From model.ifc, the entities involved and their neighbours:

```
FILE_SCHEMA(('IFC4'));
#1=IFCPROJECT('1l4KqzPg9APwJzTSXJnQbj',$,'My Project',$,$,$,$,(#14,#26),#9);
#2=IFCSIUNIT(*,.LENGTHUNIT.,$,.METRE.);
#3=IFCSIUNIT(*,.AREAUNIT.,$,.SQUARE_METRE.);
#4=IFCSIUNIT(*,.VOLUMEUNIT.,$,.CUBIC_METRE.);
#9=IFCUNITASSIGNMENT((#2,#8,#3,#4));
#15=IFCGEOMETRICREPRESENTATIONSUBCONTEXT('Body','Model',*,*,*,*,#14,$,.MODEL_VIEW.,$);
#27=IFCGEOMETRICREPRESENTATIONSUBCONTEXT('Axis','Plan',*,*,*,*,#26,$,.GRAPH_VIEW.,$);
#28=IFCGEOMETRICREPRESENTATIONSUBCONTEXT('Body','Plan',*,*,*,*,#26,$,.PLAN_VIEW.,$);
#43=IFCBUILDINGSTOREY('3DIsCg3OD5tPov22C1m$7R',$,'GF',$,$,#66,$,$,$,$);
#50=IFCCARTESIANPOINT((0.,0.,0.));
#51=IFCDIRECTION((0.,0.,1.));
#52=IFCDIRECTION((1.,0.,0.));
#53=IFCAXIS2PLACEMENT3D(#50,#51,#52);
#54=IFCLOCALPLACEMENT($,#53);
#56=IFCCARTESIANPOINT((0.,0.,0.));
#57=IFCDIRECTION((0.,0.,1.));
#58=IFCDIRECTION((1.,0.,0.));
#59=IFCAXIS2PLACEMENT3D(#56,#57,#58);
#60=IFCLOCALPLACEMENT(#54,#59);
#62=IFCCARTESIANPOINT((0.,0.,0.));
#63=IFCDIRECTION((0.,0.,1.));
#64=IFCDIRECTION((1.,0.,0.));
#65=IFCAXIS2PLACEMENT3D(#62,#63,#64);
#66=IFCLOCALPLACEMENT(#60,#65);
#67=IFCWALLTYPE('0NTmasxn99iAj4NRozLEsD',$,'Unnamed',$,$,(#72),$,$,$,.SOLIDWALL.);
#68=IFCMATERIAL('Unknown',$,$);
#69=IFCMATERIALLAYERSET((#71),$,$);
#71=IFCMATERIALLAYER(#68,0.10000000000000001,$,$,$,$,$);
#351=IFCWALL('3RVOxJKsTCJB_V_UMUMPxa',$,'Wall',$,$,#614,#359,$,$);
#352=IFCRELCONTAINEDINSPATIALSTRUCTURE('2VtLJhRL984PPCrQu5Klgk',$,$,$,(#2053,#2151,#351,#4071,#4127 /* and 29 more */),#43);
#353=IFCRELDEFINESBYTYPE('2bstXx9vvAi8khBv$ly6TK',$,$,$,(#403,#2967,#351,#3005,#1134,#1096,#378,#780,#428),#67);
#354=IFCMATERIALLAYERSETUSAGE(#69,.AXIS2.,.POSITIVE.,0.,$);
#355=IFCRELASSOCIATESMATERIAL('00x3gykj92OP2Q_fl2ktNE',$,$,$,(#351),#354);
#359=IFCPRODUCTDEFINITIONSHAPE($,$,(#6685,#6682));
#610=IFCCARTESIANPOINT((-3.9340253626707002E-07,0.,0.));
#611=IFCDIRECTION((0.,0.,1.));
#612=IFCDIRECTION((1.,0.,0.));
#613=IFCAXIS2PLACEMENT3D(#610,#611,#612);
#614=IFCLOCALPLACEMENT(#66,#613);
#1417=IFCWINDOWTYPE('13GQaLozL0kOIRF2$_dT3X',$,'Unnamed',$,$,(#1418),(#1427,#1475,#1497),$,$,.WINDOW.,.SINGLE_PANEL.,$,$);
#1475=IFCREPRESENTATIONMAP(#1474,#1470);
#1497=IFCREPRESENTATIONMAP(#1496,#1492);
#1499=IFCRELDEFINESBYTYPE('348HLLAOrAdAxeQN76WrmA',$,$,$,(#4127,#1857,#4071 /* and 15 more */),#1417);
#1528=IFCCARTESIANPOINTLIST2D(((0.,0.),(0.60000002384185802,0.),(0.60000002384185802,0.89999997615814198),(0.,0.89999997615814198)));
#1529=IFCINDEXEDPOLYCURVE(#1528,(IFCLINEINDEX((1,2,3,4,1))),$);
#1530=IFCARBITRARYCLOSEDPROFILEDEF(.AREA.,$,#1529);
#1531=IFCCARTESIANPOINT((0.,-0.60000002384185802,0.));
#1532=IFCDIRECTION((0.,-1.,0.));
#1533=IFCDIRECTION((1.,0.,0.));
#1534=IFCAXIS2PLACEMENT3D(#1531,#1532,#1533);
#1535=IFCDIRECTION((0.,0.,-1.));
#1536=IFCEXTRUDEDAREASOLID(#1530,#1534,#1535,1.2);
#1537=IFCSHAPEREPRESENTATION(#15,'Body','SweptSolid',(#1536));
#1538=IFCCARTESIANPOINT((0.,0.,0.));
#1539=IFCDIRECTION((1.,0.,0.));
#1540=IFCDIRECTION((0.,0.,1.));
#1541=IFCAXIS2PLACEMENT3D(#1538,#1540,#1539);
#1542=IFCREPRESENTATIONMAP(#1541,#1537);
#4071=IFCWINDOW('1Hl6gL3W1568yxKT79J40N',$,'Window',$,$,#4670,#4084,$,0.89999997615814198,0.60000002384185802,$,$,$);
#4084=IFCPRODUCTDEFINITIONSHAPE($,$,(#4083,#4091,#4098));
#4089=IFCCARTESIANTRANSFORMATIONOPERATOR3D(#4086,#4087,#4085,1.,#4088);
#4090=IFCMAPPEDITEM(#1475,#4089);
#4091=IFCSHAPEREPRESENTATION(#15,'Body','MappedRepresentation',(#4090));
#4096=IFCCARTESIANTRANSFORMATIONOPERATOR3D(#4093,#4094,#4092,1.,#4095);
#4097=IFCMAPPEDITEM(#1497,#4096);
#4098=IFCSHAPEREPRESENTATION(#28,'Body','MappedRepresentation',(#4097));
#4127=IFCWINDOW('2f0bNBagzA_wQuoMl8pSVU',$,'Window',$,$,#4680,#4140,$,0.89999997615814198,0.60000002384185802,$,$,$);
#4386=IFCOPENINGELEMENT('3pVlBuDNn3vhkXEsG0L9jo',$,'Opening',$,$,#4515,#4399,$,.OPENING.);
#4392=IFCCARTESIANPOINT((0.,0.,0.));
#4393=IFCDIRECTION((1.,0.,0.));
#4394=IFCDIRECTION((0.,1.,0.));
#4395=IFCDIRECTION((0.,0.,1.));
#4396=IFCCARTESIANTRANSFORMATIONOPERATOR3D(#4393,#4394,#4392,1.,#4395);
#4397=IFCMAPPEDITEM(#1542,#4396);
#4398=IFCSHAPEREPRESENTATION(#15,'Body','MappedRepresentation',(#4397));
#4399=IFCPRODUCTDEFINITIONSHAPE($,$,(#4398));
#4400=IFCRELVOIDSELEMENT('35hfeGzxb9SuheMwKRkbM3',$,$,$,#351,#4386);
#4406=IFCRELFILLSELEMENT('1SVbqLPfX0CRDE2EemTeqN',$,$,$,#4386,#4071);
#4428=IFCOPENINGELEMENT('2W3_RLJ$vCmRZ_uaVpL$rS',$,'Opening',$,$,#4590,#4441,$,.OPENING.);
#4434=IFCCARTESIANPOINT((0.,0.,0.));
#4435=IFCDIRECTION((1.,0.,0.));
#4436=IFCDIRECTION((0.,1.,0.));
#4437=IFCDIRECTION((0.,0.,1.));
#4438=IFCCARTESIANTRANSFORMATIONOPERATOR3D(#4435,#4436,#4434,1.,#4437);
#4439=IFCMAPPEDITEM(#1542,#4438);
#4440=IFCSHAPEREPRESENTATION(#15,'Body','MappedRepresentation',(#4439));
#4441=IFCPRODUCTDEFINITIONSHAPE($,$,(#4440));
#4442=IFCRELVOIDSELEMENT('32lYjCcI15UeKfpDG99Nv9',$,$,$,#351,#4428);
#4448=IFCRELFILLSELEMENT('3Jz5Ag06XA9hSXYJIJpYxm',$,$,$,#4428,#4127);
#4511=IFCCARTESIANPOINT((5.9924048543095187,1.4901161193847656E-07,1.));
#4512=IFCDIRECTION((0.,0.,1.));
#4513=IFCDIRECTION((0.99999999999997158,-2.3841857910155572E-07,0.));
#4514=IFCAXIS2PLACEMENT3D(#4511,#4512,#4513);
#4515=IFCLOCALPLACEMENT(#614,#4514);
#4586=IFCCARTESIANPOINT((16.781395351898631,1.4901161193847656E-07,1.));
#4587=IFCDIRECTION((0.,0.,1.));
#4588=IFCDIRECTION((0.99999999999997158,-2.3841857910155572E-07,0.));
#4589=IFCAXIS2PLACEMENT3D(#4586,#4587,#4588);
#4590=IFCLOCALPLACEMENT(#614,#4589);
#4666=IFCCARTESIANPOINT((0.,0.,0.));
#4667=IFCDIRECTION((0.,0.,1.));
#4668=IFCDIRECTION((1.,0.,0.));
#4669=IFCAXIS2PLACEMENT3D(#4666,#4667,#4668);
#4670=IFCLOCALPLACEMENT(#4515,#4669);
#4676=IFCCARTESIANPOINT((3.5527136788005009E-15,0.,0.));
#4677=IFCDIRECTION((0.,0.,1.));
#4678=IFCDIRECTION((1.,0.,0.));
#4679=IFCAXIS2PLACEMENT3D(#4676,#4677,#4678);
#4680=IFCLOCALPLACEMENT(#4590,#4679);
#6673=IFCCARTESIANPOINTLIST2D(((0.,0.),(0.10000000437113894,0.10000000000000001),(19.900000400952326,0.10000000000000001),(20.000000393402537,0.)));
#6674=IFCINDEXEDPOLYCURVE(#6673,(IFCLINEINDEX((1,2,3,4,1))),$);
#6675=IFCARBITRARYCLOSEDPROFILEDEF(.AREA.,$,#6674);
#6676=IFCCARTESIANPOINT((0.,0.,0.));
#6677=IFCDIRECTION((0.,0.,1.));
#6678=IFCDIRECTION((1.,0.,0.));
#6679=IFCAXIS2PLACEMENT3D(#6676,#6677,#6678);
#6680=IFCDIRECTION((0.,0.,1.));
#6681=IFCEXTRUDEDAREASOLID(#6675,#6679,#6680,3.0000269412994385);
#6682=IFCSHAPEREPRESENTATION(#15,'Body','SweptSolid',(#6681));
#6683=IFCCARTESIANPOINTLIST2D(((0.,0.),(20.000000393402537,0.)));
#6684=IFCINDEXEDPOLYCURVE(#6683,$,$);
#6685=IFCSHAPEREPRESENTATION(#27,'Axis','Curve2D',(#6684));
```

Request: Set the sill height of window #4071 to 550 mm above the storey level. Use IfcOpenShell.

```python
import numpy as np
import ifcopenshell
import ifcopenshell.api.geometry
import ifcopenshell.geom
import ifcopenshell.util.element
import ifcopenshell.util.placement
import ifcopenshell.util.shape
import ifcopenshell.util.unit

model = ifcopenshell.open("model.ifc")
unit_scale = ifcopenshell.util.unit.calculate_unit_scale(model)

window = model.by_guid("1Hl6gL3W1568yxKT79J40N")
opening = window.FillsVoids[0].RelatingOpeningElement
storey = ifcopenshell.util.element.get_container(window, ifc_class="IfcBuildingStorey")
level = ifcopenshell.util.placement.get_local_placement(storey.ObjectPlacement)[2, 3]

# The opening's origin need not be at the sill, so measure its lowest point.
shape = ifcopenshell.geom.create_shape(ifcopenshell.geom.settings(), opening)
bottom = ifcopenshell.util.shape.get_shape_bottom_elevation(shape, shape.geometry) / unit_scale
dz = level + 0.55 - bottom

shift = np.array([0.0, 0.0, dz])
# The window is placed relative to its opening, so it follows when the opening moves.
matrix = ifcopenshell.util.placement.get_local_placement(opening.ObjectPlacement)
matrix[:3, 3] += shift
ifcopenshell.api.geometry.edit_object_placement(
    model, product=opening, matrix=matrix, is_si=False, should_transform_children=True
)

print(f"moved by {dz * unit_scale:+.3f} m")

model.write("model_rev.ifc")
```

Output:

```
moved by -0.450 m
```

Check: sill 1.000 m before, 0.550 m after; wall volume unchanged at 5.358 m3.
